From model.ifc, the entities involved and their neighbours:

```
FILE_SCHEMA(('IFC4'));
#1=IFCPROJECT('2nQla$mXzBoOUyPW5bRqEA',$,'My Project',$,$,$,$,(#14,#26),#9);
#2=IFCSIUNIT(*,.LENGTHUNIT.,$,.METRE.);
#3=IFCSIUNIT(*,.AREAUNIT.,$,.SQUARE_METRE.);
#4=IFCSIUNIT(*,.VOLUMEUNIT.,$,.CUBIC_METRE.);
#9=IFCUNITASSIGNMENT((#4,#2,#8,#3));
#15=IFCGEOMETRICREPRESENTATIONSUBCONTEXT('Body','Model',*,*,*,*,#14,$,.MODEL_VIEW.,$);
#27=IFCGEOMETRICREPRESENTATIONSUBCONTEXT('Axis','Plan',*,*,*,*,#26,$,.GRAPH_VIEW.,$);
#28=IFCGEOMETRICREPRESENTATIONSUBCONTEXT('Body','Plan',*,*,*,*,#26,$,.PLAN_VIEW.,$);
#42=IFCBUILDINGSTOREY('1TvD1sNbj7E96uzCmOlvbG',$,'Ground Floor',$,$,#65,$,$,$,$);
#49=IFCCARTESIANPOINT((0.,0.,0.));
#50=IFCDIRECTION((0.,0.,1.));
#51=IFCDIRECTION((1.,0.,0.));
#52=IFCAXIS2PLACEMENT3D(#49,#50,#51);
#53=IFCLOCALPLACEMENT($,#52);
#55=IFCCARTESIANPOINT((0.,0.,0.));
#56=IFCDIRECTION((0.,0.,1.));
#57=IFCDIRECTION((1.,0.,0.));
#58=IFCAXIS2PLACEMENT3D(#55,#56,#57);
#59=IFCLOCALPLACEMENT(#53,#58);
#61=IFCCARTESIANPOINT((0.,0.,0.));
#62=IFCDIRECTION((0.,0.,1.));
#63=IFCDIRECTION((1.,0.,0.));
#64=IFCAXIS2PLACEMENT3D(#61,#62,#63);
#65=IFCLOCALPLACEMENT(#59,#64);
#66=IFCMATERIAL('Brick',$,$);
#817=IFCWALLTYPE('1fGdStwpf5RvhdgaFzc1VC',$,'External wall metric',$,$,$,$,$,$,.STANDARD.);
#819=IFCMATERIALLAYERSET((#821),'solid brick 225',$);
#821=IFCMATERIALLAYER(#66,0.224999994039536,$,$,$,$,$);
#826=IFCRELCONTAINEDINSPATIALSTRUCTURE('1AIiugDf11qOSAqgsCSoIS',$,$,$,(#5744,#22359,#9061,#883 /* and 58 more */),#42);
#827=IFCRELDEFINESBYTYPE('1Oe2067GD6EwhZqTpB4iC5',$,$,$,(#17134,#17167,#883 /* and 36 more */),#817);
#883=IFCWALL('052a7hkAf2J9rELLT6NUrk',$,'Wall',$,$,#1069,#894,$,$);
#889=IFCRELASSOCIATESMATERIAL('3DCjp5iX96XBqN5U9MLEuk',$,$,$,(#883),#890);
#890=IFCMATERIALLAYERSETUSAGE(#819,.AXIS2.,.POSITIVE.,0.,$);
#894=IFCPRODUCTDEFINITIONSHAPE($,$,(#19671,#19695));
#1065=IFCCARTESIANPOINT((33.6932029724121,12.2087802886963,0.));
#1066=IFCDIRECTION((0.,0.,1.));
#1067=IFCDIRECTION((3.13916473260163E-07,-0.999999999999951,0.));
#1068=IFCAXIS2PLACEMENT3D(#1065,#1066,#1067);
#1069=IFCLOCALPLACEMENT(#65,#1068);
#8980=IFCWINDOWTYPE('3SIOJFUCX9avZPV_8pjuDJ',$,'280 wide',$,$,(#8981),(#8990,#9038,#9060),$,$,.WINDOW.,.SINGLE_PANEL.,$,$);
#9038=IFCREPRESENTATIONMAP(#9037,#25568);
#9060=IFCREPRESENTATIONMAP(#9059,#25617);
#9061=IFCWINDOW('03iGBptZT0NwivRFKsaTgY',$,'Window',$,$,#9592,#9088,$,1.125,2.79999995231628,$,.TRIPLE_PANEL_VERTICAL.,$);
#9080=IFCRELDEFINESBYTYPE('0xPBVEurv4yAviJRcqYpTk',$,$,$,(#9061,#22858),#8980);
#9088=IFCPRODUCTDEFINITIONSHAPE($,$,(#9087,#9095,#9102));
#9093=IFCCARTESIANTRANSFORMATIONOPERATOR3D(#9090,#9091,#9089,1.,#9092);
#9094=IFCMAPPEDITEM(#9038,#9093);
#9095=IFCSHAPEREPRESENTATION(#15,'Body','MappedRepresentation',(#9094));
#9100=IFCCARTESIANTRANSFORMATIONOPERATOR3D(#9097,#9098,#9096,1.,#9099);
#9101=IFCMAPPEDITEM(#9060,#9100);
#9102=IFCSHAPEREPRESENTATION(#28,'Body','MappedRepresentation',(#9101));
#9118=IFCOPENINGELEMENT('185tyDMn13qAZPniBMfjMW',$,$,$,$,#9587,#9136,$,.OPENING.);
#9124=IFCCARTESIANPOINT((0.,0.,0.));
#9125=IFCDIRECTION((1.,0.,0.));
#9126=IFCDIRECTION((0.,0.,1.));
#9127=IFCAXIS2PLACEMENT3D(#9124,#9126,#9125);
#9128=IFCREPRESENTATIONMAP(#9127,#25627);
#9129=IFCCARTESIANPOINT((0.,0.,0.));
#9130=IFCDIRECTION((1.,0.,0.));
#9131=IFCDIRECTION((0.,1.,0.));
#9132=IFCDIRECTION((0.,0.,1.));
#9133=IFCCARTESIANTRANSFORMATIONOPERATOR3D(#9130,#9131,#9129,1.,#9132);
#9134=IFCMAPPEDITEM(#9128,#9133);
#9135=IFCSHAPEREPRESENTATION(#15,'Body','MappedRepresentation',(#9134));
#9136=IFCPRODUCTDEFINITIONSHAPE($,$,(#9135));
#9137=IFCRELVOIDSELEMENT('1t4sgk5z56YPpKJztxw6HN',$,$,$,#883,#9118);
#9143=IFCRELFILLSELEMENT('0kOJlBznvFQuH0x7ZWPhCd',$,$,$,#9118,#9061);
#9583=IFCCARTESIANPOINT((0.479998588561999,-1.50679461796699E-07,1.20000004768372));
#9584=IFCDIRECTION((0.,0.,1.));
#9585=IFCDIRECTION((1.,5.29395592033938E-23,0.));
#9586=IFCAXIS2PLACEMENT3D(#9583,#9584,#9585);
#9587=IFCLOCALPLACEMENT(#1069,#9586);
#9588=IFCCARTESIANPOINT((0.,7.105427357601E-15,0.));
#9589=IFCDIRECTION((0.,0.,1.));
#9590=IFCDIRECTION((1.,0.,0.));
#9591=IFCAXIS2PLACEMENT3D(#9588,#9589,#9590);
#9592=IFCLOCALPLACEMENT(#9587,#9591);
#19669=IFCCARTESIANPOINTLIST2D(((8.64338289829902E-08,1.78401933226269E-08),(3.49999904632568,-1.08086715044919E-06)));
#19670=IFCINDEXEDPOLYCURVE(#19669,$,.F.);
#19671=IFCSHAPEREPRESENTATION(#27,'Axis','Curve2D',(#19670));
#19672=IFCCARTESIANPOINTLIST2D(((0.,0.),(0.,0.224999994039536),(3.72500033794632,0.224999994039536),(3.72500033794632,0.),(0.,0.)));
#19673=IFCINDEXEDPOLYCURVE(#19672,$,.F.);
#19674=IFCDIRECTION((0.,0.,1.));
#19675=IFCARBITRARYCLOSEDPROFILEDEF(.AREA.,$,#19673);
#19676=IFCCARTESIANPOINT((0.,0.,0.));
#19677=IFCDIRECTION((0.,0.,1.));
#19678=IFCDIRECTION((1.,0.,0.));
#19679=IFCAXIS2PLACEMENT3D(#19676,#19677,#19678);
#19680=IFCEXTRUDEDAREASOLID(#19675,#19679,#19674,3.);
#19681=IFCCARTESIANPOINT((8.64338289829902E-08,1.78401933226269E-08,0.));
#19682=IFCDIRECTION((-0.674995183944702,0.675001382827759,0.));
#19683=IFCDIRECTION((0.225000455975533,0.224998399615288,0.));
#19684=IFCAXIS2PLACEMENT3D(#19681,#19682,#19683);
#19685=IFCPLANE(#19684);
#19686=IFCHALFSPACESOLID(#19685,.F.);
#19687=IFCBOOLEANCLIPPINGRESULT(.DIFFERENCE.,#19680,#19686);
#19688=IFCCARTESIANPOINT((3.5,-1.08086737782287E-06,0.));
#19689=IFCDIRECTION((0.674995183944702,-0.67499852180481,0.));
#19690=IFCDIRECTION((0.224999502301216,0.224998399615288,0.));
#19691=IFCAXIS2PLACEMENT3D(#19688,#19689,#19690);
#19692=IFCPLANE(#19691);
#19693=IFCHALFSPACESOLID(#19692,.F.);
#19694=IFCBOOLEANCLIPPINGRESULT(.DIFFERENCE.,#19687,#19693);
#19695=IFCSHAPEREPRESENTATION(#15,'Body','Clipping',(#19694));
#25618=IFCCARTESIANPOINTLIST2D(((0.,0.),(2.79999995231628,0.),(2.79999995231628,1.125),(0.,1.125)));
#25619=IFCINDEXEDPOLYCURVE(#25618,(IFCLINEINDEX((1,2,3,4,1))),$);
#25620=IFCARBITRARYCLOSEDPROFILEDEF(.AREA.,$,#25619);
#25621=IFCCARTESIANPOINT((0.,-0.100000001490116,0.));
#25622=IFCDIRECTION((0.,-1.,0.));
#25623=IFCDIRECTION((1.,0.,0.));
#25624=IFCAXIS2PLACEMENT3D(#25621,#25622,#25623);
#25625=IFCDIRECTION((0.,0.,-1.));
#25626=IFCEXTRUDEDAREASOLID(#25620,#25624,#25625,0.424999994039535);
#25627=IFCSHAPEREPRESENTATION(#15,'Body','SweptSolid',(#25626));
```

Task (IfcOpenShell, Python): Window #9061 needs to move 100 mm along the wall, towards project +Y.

```python
import ifcopenshell
import ifcopenshell.api.geometry
import ifcopenshell.util.placement
import ifcopenshell.util.unit

model = ifcopenshell.open("model.ifc")
unit_scale = ifcopenshell.util.unit.calculate_unit_scale(model)

window = model.by_id(9061)
opening = window.FillsVoids[0].RelatingOpeningElement
wall = opening.VoidsElements[0].RelatingBuildingElement

wall_matrix = ifcopenshell.util.placement.get_local_placement(wall.ObjectPlacement)
shift = wall_matrix[:3, 0] * -0.1 / unit_scale
before = ifcopenshell.util.placement.get_local_placement(window.ObjectPlacement)[:3, 3].copy()

# The window is placed relative to its opening, so it follows when the opening moves.
matrix = ifcopenshell.util.placement.get_local_placement(opening.ObjectPlacement)
matrix[:3, 3] += shift
ifcopenshell.api.geometry.edit_object_placement(
    model, product=opening, matrix=matrix, is_si=False, should_transform_children=True
)

after = ifcopenshell.util.placement.get_local_placement(window.ObjectPlacement)[:3, 3]
print("window moved by", (after - before).round(3) + 0.0)

model.write("model-out.ifc")
```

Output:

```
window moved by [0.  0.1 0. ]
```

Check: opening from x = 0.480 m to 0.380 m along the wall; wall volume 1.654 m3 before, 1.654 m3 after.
